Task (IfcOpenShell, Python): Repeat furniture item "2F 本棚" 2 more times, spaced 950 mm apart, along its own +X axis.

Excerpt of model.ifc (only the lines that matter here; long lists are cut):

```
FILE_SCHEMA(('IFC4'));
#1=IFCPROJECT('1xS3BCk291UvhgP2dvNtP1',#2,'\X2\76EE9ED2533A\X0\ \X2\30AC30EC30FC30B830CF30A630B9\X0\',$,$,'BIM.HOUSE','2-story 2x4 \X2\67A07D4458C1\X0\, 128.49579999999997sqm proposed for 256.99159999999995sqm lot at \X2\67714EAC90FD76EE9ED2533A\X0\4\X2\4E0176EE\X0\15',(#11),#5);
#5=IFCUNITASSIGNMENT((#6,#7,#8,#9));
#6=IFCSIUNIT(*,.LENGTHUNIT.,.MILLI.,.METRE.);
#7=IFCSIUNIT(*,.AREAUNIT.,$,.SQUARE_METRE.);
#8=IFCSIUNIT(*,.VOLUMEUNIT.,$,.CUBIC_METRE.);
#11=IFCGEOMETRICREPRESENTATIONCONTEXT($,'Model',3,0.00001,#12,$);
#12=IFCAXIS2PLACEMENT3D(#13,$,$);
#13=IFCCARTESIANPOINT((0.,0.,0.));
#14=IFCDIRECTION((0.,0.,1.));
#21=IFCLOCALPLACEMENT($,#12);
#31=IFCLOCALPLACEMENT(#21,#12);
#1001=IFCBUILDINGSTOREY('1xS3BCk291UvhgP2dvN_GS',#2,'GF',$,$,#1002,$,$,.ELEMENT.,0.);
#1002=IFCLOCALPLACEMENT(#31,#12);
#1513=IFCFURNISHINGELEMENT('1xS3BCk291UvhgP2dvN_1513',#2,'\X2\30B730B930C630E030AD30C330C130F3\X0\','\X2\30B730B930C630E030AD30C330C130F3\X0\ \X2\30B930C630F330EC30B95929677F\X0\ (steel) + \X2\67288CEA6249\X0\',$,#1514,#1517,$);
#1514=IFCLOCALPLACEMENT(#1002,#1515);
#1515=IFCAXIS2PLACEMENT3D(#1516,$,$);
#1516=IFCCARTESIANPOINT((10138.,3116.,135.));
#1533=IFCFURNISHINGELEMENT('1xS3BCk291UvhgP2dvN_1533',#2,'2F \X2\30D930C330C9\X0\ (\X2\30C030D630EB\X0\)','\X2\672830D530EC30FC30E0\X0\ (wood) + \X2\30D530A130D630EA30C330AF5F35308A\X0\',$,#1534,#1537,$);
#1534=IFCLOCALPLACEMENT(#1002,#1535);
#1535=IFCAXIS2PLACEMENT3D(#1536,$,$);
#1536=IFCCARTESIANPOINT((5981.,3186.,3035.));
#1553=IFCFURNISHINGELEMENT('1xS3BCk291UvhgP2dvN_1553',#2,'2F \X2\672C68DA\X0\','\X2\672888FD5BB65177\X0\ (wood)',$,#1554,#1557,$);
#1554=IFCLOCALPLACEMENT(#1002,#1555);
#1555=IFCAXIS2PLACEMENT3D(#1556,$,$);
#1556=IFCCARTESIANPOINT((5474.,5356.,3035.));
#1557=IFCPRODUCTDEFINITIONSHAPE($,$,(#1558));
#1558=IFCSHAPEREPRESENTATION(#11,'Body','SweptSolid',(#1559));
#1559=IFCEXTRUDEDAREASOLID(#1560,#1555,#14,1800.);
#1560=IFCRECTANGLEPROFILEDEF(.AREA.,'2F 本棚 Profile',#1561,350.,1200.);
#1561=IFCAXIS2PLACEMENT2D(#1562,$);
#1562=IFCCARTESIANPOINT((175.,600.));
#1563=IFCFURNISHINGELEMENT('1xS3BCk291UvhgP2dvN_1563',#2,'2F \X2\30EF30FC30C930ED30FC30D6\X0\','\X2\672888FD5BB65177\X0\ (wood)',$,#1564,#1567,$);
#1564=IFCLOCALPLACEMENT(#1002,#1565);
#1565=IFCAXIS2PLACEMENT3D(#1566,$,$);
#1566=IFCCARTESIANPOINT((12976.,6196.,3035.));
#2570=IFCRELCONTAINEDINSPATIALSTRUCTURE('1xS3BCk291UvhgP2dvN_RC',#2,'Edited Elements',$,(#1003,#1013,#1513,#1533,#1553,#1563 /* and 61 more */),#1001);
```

```python
import ifcopenshell
import ifcopenshell.api.geometry
import ifcopenshell.api.root
import ifcopenshell.util.element
import ifcopenshell.util.placement
import ifcopenshell.util.unit

model = ifcopenshell.open("model.ifc")
unit_scale = ifcopenshell.util.unit.calculate_unit_scale(model)


def reuse_history(source, copy):
    """copy_class also copies each property set's owner history, people and application; keep the originals."""
    for rel in copy.IsDefinedBy:
        if rel.is_a("IfcRelDefinesByProperties") and (history := rel.RelatingPropertyDefinition.OwnerHistory):
            rel.RelatingPropertyDefinition.OwnerHistory = source.OwnerHistory
            ifcopenshell.util.element.remove_deep2(model, history)


source = model.by_guid("1xS3BCk291UvhgP2dvN_1553")
base = ifcopenshell.util.placement.get_local_placement(source.ObjectPlacement)
step = base[:3, 0] * 0.95 / unit_scale

for i in range(1, 3):
    copy = ifcopenshell.api.root.copy_class(model, product=source)
    copy.Representation = ifcopenshell.util.element.copy_deep(
        model, source.Representation, exclude=["IfcGeometricRepresentationContext", "IfcRepresentationMap"]
    )
    reuse_history(source, copy)
    matrix = base.copy()
    matrix[:3, 3] += i * step
    print("added at", matrix[:3, 3].round(3) + 0.0)
    ifcopenshell.api.geometry.edit_object_placement(model, product=copy, matrix=matrix, is_si=False)

model.write("model-out.ifc")
```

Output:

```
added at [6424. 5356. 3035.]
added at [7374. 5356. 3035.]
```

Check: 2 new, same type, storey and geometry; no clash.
